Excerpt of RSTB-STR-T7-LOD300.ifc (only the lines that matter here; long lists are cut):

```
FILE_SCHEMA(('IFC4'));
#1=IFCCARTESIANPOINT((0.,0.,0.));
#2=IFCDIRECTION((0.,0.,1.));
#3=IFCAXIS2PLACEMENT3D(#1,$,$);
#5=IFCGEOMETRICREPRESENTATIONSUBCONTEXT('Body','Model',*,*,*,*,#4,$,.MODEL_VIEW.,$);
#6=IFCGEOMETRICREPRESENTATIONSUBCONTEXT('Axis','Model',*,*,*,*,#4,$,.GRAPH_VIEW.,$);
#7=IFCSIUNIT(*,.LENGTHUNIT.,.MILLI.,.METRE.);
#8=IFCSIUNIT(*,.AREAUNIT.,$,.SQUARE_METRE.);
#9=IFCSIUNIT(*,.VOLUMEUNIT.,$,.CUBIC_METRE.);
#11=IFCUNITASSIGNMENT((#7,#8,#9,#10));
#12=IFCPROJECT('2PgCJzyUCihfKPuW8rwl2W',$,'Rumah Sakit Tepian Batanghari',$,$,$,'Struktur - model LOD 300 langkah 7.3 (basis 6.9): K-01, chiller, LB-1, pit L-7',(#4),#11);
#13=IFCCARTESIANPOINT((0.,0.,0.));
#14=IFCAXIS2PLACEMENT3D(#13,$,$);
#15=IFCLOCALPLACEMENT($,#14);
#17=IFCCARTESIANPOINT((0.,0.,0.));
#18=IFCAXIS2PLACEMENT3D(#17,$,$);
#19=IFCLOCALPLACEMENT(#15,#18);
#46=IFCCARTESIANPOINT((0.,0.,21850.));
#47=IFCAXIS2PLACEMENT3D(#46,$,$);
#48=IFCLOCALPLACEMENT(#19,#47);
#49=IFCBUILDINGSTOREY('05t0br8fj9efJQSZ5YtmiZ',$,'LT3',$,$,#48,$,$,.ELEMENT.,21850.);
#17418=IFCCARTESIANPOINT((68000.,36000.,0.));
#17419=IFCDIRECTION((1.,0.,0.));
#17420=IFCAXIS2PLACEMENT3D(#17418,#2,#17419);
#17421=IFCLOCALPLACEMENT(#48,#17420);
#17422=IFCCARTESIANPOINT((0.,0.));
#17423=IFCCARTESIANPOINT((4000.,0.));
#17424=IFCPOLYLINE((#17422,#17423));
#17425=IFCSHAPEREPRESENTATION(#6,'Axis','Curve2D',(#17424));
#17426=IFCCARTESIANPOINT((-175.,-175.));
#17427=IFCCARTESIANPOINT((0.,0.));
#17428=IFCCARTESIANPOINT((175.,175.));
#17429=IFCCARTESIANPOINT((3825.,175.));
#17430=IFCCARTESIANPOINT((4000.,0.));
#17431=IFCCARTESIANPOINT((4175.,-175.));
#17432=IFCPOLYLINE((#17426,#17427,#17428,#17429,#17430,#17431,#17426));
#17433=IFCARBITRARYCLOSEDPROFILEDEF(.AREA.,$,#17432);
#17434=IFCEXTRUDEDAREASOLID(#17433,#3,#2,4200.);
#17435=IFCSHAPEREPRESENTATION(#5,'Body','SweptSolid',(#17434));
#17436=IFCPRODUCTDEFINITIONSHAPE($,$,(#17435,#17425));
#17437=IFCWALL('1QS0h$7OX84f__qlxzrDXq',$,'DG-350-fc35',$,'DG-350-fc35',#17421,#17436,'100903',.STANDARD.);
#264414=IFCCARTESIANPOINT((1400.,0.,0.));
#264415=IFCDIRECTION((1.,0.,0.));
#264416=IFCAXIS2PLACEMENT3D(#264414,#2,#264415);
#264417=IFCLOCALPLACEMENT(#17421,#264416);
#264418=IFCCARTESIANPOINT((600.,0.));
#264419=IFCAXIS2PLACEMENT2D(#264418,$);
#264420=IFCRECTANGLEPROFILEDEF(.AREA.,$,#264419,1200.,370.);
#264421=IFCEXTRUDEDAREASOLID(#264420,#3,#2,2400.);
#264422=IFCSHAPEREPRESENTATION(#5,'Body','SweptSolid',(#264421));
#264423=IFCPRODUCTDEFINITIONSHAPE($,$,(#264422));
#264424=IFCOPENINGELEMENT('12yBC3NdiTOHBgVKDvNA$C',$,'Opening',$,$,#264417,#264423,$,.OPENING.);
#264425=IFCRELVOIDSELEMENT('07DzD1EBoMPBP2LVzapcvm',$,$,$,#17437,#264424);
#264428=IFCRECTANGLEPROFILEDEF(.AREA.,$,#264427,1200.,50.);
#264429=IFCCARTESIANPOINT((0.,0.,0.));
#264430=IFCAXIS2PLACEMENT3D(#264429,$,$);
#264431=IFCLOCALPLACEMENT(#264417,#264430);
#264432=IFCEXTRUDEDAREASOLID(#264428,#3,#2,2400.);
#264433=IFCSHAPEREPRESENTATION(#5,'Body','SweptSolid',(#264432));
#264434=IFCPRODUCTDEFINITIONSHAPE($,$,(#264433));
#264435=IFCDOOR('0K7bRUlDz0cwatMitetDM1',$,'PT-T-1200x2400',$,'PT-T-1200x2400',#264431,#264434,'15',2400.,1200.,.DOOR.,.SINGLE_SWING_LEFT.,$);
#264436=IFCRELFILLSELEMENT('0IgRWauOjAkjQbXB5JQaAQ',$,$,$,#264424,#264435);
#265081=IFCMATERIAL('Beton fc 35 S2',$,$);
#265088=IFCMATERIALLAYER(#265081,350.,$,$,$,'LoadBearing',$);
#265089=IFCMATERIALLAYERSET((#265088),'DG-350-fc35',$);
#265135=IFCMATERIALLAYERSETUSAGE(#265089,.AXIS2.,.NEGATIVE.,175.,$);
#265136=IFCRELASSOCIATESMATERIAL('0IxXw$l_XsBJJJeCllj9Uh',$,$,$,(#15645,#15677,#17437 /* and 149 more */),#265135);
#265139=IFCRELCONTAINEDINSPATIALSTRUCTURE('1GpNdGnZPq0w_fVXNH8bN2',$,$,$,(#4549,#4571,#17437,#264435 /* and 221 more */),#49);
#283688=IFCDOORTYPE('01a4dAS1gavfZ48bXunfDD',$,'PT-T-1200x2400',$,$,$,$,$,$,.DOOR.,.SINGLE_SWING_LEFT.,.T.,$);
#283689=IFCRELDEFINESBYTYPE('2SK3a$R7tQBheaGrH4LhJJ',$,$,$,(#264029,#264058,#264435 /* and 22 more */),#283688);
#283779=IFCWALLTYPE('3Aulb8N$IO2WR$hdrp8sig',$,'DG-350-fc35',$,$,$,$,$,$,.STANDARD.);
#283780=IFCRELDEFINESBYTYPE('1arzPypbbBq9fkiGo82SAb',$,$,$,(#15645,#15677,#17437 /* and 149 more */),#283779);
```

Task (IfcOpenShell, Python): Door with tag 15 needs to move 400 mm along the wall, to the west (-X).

```python
import ifcopenshell
import ifcopenshell.api.geometry
import ifcopenshell.util.placement
import ifcopenshell.util.unit

model = ifcopenshell.open("RSTB-STR-T7-LOD300.ifc")
unit_scale = ifcopenshell.util.unit.calculate_unit_scale(model)

door = model.by_guid("0K7bRUlDz0cwatMitetDM1")
opening = door.FillsVoids[0].RelatingOpeningElement
wall = opening.VoidsElements[0].RelatingBuildingElement

wall_matrix = ifcopenshell.util.placement.get_local_placement(wall.ObjectPlacement)
shift = wall_matrix[:3, 0] * -0.4 / unit_scale
before = ifcopenshell.util.placement.get_local_placement(door.ObjectPlacement)[:3, 3].copy()

# The door is placed relative to its opening, so it follows when the opening moves.
matrix = ifcopenshell.util.placement.get_local_placement(opening.ObjectPlacement)
matrix[:3, 3] += shift
ifcopenshell.api.geometry.edit_object_placement(
    model, product=opening, matrix=matrix, is_si=False, should_transform_children=True
)

after = ifcopenshell.util.placement.get_local_placement(door.ObjectPlacement)[:3, 3]
print("door moved by", (after - before).round(3) + 0.0)

model.write("RSTB-STR-T7-LOD300-out.ifc")
```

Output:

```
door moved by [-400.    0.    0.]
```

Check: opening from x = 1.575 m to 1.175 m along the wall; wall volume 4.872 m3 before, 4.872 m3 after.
